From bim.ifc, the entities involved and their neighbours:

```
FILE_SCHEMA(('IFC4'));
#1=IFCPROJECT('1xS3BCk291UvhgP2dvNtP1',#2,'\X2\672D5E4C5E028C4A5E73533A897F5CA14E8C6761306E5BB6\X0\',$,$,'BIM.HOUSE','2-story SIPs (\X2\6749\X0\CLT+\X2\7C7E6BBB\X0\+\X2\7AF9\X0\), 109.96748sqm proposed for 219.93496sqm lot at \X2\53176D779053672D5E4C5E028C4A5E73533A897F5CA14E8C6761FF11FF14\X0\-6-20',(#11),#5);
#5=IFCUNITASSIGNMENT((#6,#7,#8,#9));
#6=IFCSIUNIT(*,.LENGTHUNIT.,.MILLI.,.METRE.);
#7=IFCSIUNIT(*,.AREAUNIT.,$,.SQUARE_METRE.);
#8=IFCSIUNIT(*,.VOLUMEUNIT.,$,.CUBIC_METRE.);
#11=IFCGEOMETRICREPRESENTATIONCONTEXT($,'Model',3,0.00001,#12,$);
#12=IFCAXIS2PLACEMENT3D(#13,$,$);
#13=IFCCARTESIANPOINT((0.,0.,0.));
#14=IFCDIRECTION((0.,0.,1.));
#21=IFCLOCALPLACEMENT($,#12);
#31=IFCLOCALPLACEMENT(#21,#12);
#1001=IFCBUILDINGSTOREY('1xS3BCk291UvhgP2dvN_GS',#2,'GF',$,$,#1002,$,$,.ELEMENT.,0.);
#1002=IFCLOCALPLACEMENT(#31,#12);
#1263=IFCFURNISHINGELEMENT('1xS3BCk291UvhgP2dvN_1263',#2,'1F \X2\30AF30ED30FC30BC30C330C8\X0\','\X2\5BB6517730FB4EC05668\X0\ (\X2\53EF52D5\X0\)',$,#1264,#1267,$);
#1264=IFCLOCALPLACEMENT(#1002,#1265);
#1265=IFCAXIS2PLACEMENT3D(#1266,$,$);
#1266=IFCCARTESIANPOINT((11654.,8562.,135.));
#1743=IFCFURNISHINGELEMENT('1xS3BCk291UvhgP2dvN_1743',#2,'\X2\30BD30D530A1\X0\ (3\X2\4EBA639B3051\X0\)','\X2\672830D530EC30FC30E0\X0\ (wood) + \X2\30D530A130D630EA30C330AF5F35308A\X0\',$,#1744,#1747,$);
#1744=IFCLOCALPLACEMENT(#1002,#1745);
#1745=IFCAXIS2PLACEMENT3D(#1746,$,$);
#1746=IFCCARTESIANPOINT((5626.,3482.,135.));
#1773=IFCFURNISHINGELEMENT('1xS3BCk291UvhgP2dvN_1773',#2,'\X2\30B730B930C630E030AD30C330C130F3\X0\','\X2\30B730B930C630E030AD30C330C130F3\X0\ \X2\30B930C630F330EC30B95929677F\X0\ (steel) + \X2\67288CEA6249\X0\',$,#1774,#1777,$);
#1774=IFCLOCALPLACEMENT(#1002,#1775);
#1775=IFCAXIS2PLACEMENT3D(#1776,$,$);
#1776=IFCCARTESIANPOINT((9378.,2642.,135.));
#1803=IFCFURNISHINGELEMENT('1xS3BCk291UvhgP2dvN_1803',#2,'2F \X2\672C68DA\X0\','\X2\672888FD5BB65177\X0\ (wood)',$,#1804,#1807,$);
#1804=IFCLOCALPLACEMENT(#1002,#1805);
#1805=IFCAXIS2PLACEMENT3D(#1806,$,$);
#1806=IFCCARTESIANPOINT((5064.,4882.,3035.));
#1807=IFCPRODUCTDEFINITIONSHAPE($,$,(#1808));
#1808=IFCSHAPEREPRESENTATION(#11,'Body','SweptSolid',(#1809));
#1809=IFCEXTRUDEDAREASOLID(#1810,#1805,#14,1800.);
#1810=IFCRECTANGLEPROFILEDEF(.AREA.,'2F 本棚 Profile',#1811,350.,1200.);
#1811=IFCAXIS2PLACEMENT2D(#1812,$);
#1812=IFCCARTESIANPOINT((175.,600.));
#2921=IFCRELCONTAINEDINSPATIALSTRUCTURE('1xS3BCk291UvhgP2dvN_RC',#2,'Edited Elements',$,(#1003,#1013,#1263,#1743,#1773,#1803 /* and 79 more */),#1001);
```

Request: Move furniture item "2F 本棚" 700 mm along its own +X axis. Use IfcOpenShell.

```python
import ifcopenshell
import ifcopenshell.api.geometry
import ifcopenshell.util.placement

model = ifcopenshell.open("bim.ifc")

item = model.by_guid("1xS3BCk291UvhgP2dvN_1803")
matrix = ifcopenshell.util.placement.get_local_placement(item.ObjectPlacement)
matrix[:3, 3] += matrix[:3, 0] * 700.0
ifcopenshell.api.geometry.edit_object_placement(model, product=item, matrix=matrix, is_si=False)

print(ifcopenshell.util.placement.get_local_placement(item.ObjectPlacement).round(3) + 0.0)

model.write("bim-out.ifc")
```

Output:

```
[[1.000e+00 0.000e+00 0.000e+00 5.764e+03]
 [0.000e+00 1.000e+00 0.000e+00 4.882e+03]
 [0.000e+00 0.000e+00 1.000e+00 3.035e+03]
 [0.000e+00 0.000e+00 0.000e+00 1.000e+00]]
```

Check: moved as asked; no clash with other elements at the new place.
